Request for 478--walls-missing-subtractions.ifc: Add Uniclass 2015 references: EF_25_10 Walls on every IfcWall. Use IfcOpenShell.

First a look at what the model holds.

```python
import ifcopenshell

model = ifcopenshell.open("478--walls-missing-subtractions.ifc")
print(model.schema)
print("classifications:", [c.Name for c in model.by_type("IfcClassification")])
for ifc_class in ("IfcDoor", "IfcRoof", "IfcStair", "IfcWall", "IfcWindow"):
    print(ifc_class, len(model.by_type(ifc_class)))
```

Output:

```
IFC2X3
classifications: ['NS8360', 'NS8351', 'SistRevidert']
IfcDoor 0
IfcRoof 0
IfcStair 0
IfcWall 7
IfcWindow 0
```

```python
import ifcopenshell
import ifcopenshell.api.classification

model = ifcopenshell.open("478--walls-missing-subtractions.ifc")

# IFC2X3 requires Source and Edition and has no link from the project to the system.
system = model.create_entity("IfcClassification", Source="NBS", Edition="2015", Name="Uniclass 2015")

codes = {
    "IfcWall": ("EF_25_10", "Walls"),
}
for ifc_class, (code, name) in codes.items():
    products = model.by_type(ifc_class)
    ifcopenshell.api.classification.add_reference(
        model, products=products, classification=system, identification=code, name=name
    )
    print(code, len(products))

model.write("478--walls-missing-subtractions_updated.ifc")
```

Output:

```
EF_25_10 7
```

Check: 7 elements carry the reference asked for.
